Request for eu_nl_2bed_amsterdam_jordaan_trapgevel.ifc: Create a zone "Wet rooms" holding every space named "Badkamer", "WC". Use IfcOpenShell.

First a look at what the model holds.

```python
import ifcopenshell

model = ifcopenshell.open("eu_nl_2bed_amsterdam_jordaan_trapgevel.ifc")
print(model.schema)
seen = {}
for space in model.by_type("IfcSpace"):
    seen[space.LongName] = seen.get(space.LongName, 0) + 1
for name, count in sorted(seen.items(), key=str):
    print(count, "x", name)
print("zones:", [z.Name for z in model.by_type("IfcZone")][:20])
```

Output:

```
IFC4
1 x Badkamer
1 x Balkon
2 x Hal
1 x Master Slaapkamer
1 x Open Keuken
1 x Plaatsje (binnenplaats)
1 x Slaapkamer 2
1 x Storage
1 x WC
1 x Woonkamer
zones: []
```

```python
import ifcopenshell
import ifcopenshell.api.group
import ifcopenshell.api.root

model = ifcopenshell.open("eu_nl_2bed_amsterdam_jordaan_trapgevel.ifc")

names = {"Badkamer", "WC"}
spaces = [s for s in model.by_type("IfcSpace") if s.LongName in names]

zone = ifcopenshell.api.root.create_entity(model, ifc_class="IfcZone", name="Wet rooms")
ifcopenshell.api.group.assign_group(model, products=spaces, group=zone)
print(len(spaces), "spaces in", zone.Name)

model.write("eu_nl_2bed_amsterdam_jordaan_trapgevel_edited.ifc")
```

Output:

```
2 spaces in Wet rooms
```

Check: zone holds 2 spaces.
